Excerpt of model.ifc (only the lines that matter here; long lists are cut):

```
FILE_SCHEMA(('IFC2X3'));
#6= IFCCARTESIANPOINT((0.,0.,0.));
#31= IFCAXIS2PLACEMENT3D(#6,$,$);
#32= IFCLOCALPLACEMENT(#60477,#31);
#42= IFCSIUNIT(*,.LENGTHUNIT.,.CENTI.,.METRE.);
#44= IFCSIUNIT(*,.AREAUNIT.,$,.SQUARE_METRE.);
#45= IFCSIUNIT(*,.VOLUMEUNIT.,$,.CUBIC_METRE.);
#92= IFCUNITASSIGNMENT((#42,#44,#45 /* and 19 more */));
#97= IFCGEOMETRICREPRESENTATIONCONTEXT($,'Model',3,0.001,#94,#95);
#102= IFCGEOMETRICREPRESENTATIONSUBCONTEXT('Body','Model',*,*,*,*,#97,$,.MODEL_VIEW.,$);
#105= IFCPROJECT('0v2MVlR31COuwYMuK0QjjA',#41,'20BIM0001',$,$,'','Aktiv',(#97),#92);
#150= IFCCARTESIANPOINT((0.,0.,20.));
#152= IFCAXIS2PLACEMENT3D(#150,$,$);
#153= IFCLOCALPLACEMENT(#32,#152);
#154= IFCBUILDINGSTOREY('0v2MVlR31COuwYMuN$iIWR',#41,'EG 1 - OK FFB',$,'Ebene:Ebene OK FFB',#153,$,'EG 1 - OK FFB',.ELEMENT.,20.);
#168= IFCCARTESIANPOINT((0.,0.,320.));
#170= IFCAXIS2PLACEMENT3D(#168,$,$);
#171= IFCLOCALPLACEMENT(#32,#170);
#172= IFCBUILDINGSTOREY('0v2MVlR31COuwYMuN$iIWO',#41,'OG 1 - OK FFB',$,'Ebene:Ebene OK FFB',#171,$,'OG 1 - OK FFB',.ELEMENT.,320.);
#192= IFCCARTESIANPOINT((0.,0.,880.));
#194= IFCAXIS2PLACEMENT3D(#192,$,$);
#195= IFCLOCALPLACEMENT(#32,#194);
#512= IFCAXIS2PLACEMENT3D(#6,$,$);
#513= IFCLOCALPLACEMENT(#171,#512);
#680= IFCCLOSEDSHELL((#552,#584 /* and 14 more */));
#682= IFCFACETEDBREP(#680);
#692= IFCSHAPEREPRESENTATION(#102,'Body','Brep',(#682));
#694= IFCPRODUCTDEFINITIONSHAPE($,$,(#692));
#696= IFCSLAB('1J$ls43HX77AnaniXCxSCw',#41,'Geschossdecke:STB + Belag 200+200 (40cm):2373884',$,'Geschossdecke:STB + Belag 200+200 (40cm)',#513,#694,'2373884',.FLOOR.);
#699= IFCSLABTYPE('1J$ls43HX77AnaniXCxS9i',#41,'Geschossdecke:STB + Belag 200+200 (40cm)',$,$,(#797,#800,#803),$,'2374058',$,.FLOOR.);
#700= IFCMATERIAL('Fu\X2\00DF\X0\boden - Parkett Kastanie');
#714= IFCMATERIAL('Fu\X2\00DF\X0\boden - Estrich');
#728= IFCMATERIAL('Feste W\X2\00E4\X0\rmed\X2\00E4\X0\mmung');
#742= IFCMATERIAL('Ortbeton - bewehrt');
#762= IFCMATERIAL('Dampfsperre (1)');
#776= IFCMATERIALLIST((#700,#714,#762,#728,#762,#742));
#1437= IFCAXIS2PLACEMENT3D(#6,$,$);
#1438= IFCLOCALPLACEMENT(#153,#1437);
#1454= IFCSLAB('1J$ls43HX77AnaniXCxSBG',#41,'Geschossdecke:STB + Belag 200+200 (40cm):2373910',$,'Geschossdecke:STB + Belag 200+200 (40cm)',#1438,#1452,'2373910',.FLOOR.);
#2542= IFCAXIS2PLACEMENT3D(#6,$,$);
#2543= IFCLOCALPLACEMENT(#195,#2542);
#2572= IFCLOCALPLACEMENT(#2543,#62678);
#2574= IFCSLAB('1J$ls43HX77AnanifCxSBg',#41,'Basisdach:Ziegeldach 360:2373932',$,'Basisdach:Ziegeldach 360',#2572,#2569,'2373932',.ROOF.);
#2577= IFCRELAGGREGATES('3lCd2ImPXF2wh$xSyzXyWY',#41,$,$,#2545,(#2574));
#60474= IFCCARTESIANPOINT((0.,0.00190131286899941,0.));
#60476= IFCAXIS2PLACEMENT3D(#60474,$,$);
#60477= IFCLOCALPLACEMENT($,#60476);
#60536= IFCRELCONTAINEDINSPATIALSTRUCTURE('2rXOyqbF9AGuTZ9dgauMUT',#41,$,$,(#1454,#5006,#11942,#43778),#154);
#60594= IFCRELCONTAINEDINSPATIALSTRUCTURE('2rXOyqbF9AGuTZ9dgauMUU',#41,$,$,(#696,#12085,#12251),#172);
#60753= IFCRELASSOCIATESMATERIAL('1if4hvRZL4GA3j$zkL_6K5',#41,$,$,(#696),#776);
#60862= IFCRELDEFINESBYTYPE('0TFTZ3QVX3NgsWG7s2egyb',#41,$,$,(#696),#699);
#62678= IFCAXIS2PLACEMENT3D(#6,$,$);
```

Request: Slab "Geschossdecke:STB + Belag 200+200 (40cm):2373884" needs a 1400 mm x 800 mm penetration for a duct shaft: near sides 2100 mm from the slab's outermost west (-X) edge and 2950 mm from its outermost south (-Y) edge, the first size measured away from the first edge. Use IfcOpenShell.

```python
import numpy as np
import ifcopenshell
import ifcopenshell.api.feature
import ifcopenshell.api.geometry
import ifcopenshell.api.root
import ifcopenshell.geom
import ifcopenshell.util.placement
import ifcopenshell.util.representation
import ifcopenshell.util.shape
import ifcopenshell.util.unit

model = ifcopenshell.open("model.ifc")
unit_scale = ifcopenshell.util.unit.calculate_unit_scale(model)
settings = ifcopenshell.geom.settings()


def volume(element):
    """Net volume in cubic metres, openings subtracted."""
    shape = ifcopenshell.geom.create_shape(settings, element)
    return ifcopenshell.util.shape.get_volume(shape.geometry)


slab = model.by_id(696)
before = volume(slab)

# Extent in the slab's own axes, in metres. The edges named are its -X and -Y sides.
slab_shape = ifcopenshell.geom.create_shape(settings, slab)
vertices = ifcopenshell.util.shape.get_vertices(slab_shape.geometry)
x_min, y_min, bottom = vertices.min(axis=0)
top = vertices[:, 2].max()

opening = ifcopenshell.api.root.create_entity(model, ifc_class="IfcOpeningElement", name="Duct shaft opening")
context = ifcopenshell.util.representation.get_context(model, "Model", "Body", "MODEL_VIEW")
width, depth = 1.4, 0.8
outline = [(0.0, 0.0), (width, 0.0), (width, depth), (0.0, depth), (0.0, 0.0)]
# Overshoot both faces by 50 mm so the cut is clean.
shape = ifcopenshell.api.geometry.add_slab_representation(
    model, context=context, depth=top - bottom + 0.1, polyline=outline
)
ifcopenshell.api.geometry.assign_representation(model, product=opening, representation=shape)

matrix = ifcopenshell.util.placement.get_local_placement(slab.ObjectPlacement)
matrix[:, 3] = matrix @ np.append(np.array([x_min + 2.1, y_min + 2.95, bottom - 0.05]) / unit_scale, 1.0)
ifcopenshell.api.geometry.edit_object_placement(model, product=opening, matrix=matrix, is_si=False)
ifcopenshell.api.feature.add_feature(model, feature=opening, element=slab)

after = volume(slab)

print(f"slab volume {before:.3f} -> {after:.3f} m3")

model.write("model_v2.ifc")
```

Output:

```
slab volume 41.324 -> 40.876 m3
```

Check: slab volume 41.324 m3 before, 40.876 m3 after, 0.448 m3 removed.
